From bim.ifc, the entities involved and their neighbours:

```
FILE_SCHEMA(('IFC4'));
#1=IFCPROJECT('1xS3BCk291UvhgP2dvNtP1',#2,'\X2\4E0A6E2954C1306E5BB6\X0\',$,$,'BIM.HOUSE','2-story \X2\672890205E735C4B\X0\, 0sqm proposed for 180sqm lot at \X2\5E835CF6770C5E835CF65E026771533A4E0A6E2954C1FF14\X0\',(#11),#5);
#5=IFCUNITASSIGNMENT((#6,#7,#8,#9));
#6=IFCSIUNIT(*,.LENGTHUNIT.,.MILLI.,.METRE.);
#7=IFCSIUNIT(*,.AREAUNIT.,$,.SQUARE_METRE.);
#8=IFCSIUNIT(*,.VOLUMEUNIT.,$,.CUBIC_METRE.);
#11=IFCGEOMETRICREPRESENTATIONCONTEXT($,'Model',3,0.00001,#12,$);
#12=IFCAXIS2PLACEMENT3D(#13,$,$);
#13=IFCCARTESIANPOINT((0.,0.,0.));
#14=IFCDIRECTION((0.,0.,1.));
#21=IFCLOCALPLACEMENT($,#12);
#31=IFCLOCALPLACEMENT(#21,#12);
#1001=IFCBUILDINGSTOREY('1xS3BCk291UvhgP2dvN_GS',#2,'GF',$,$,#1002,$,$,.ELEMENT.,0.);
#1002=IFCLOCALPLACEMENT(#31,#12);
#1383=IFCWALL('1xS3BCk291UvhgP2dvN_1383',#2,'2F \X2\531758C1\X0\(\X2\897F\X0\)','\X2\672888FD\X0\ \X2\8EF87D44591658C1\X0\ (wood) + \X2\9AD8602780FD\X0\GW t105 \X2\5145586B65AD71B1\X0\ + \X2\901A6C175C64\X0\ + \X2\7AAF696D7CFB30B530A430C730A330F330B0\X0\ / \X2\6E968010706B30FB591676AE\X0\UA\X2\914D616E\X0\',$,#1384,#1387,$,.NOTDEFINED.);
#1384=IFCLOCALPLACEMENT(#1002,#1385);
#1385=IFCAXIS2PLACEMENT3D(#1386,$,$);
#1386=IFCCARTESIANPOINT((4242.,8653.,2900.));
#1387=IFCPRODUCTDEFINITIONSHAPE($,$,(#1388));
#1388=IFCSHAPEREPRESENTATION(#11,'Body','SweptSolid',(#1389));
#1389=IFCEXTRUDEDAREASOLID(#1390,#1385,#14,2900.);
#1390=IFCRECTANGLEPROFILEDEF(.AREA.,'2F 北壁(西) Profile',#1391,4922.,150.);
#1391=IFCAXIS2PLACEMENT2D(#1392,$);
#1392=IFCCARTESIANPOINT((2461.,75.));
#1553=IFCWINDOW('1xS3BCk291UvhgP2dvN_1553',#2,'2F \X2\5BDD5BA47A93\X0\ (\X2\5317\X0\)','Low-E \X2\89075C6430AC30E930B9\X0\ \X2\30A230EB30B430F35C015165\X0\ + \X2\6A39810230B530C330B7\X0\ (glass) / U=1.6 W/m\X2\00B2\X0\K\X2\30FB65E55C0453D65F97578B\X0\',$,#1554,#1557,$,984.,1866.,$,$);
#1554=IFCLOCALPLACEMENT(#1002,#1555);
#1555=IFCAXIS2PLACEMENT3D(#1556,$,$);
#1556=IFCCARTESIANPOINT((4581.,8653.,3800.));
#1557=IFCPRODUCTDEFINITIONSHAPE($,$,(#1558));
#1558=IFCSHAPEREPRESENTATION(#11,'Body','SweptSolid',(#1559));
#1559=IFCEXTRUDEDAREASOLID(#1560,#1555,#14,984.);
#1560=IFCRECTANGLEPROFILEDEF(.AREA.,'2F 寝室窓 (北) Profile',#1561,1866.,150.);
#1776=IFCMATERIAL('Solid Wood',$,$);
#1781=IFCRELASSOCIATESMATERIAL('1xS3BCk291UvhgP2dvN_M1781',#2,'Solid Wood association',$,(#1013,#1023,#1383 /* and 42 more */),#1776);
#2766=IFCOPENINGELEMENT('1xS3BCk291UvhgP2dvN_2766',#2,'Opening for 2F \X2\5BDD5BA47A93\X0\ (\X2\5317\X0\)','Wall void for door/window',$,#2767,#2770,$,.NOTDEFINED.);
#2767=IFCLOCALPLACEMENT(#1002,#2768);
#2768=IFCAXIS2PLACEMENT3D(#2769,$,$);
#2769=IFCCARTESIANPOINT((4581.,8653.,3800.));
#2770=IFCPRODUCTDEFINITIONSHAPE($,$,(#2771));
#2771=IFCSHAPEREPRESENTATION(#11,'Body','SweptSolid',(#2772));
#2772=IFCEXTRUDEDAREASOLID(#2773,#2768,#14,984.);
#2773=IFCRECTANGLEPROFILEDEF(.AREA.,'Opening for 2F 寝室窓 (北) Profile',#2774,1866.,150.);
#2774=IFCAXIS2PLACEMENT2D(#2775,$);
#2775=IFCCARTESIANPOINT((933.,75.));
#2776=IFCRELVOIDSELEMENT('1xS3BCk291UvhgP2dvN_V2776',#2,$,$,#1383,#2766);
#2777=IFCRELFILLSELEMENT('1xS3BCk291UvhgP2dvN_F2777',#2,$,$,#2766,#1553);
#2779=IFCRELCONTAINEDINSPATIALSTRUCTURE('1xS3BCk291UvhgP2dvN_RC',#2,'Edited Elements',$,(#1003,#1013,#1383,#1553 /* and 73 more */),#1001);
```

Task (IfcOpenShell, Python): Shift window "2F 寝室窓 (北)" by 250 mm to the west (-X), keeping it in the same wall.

```python
import ifcopenshell
import ifcopenshell.api.geometry
import ifcopenshell.util.placement
import ifcopenshell.util.unit

model = ifcopenshell.open("bim.ifc")
unit_scale = ifcopenshell.util.unit.calculate_unit_scale(model)

window = model.by_guid("1xS3BCk291UvhgP2dvN_1553")
opening = window.FillsVoids[0].RelatingOpeningElement
wall = opening.VoidsElements[0].RelatingBuildingElement

wall_matrix = ifcopenshell.util.placement.get_local_placement(wall.ObjectPlacement)
shift = wall_matrix[:3, 0] * -0.25 / unit_scale
before = ifcopenshell.util.placement.get_local_placement(window.ObjectPlacement)[:3, 3].copy()

# The window is not placed relative to its opening, so move both.
for product in (opening, window):
    matrix = ifcopenshell.util.placement.get_local_placement(product.ObjectPlacement)
    matrix[:3, 3] += shift
    ifcopenshell.api.geometry.edit_object_placement(model, product=product, matrix=matrix, is_si=False)

after = ifcopenshell.util.placement.get_local_placement(window.ObjectPlacement)[:3, 3]
print("window moved by", (after - before).round(3) + 0.0)

model.write("bim_edited.ifc")
```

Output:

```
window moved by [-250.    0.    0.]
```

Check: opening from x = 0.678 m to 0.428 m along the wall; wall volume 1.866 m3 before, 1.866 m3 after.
